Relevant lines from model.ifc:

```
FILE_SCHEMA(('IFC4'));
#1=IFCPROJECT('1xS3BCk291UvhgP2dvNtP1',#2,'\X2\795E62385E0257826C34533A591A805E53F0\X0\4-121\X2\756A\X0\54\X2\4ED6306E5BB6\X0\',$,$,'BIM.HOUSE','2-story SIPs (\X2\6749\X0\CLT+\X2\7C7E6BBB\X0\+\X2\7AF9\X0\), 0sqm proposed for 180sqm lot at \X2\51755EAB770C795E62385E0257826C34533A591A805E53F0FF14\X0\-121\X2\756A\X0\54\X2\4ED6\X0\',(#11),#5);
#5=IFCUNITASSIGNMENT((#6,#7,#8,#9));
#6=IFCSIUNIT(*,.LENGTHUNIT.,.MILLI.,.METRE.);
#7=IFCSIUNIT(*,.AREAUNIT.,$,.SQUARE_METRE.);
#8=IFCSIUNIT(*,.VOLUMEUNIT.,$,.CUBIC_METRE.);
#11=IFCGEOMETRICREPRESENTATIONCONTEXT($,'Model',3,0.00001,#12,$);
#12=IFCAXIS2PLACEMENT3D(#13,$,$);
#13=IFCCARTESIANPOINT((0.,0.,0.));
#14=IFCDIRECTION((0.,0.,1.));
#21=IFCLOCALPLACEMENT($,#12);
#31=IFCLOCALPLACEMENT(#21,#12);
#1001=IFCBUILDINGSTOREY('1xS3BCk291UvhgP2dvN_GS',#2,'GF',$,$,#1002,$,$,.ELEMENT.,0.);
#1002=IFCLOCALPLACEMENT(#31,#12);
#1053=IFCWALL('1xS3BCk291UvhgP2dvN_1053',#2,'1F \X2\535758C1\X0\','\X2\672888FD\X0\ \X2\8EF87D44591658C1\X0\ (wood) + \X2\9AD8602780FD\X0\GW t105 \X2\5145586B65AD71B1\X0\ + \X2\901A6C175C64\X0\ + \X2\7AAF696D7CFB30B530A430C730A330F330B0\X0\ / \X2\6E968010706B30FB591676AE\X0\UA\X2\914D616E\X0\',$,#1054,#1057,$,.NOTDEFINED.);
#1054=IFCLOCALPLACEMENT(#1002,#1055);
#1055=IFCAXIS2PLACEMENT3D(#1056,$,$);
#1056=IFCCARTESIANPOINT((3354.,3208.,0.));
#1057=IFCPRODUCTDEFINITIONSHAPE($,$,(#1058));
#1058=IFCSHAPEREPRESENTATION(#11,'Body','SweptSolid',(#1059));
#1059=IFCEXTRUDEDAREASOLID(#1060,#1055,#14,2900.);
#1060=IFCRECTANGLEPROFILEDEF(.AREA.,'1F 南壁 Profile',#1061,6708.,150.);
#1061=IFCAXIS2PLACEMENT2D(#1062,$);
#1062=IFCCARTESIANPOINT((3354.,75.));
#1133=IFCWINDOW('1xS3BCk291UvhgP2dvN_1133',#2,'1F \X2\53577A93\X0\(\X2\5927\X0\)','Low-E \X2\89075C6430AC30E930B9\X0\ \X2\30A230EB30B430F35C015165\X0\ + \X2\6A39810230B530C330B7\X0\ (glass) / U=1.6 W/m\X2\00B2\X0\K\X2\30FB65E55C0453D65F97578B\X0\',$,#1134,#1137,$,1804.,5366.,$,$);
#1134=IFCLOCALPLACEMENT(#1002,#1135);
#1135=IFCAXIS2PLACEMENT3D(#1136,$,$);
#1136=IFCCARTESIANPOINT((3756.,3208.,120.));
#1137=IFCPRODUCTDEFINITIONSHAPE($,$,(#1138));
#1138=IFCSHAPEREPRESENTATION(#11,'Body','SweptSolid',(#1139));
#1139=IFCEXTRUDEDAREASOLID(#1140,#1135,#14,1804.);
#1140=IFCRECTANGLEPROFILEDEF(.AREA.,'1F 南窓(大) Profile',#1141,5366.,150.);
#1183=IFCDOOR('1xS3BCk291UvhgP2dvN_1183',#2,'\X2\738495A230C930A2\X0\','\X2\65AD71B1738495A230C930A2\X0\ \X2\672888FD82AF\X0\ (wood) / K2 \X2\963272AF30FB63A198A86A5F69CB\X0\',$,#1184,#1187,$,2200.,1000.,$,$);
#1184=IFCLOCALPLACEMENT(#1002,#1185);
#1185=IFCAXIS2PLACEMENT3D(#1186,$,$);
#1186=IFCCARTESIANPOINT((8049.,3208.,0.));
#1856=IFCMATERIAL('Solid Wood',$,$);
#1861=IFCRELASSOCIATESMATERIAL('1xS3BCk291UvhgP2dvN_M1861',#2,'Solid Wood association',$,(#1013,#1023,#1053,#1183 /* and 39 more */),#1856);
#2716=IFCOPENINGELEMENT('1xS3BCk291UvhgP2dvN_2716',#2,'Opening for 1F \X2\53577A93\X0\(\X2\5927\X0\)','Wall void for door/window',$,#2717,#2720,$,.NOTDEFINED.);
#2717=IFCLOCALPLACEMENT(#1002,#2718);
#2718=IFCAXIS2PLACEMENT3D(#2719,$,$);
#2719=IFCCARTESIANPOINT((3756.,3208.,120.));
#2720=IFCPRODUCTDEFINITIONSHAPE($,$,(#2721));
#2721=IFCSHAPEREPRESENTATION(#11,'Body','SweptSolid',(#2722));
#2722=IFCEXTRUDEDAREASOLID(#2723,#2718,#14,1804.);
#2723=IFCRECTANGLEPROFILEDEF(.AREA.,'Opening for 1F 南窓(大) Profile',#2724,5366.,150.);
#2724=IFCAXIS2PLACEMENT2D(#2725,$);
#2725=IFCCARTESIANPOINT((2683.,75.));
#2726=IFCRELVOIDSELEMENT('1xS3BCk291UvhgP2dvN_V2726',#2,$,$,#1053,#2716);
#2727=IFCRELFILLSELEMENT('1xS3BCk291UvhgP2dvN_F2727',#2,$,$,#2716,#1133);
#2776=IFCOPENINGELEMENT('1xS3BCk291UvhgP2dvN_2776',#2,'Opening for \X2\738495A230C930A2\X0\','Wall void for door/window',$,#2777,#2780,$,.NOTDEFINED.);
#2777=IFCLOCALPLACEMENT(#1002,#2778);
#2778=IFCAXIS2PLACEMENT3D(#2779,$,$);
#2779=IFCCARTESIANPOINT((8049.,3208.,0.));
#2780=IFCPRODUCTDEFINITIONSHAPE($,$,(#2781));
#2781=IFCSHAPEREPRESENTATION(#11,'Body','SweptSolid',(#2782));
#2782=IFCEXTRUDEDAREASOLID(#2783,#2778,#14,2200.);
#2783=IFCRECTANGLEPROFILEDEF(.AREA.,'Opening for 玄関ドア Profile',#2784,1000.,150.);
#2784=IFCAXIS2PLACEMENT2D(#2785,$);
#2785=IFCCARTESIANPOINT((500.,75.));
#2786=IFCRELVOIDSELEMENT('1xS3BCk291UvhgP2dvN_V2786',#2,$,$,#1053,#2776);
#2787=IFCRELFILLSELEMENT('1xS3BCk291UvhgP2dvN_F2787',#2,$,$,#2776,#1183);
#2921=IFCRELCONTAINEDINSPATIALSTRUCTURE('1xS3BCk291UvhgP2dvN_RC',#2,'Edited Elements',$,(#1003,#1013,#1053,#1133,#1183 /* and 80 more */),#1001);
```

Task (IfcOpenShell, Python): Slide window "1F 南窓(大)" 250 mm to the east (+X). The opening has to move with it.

```python
import ifcopenshell
import ifcopenshell.api.geometry
import ifcopenshell.util.placement
import ifcopenshell.util.unit

model = ifcopenshell.open("model.ifc")
unit_scale = ifcopenshell.util.unit.calculate_unit_scale(model)

window = model.by_guid("1xS3BCk291UvhgP2dvN_1133")
opening = window.FillsVoids[0].RelatingOpeningElement
wall = opening.VoidsElements[0].RelatingBuildingElement

wall_matrix = ifcopenshell.util.placement.get_local_placement(wall.ObjectPlacement)
shift = wall_matrix[:3, 0] * 0.25 / unit_scale
before = ifcopenshell.util.placement.get_local_placement(window.ObjectPlacement)[:3, 3].copy()

# The window is not placed relative to its opening, so move both.
for product in (opening, window):
    matrix = ifcopenshell.util.placement.get_local_placement(product.ObjectPlacement)
    matrix[:3, 3] += shift
    ifcopenshell.api.geometry.edit_object_placement(model, product=product, matrix=matrix, is_si=False)

after = ifcopenshell.util.placement.get_local_placement(window.ObjectPlacement)[:3, 3]
print("window moved by", (after - before).round(3) + 0.0)

model.write("model_v2.ifc")
```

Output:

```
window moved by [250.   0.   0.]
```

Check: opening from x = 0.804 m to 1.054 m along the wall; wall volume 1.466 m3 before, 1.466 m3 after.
